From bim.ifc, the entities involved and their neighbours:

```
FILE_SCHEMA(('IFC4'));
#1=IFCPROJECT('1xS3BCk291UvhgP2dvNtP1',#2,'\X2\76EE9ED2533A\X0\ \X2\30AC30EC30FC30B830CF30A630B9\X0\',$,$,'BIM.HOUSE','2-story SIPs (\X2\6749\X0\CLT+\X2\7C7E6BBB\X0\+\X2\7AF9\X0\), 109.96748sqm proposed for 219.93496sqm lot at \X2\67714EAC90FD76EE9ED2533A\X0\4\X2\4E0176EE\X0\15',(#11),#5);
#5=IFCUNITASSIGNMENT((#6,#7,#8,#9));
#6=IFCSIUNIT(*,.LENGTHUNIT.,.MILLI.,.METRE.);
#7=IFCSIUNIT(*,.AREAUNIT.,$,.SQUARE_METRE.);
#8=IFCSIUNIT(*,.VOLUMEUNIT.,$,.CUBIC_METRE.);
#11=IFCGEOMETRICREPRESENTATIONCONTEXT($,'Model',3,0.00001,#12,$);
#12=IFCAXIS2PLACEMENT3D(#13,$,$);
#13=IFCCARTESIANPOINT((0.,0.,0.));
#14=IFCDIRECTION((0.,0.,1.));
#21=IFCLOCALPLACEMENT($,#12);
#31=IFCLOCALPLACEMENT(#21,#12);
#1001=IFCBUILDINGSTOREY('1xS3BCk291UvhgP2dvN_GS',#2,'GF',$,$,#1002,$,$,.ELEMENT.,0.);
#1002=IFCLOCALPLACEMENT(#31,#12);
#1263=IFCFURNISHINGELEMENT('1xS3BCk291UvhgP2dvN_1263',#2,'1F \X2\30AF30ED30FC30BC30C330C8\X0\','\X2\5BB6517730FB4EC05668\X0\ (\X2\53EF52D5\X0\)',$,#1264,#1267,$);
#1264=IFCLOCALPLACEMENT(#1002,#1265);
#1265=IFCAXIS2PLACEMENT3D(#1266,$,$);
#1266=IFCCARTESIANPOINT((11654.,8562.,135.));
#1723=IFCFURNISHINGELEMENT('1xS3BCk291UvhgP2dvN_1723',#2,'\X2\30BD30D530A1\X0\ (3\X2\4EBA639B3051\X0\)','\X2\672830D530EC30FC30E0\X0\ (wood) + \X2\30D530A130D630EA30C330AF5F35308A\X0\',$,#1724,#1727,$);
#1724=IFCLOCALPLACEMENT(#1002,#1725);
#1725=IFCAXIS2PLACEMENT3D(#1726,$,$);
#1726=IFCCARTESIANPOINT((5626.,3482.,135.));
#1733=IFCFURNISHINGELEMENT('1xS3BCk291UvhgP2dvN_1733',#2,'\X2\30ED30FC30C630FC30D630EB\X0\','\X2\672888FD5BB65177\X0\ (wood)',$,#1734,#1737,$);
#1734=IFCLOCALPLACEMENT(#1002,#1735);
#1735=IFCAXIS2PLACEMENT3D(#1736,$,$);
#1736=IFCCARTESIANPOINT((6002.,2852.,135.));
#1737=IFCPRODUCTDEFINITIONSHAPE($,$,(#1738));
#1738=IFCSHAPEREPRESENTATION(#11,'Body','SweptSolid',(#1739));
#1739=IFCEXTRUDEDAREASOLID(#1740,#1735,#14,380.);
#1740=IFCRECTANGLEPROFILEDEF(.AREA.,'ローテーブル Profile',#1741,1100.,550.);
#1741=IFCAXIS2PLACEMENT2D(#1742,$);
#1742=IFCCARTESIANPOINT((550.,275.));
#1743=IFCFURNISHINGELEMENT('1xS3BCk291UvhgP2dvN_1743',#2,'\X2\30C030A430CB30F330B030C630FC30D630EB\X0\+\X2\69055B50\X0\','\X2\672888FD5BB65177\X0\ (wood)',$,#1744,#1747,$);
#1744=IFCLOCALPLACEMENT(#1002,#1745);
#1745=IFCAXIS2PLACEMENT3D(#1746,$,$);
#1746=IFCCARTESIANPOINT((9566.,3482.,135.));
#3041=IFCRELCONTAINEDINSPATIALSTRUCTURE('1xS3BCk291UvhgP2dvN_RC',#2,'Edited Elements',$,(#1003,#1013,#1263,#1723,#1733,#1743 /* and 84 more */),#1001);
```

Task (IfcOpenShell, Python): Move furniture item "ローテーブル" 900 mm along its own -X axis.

```python
import ifcopenshell
import ifcopenshell.api.geometry
import ifcopenshell.util.placement

model = ifcopenshell.open("bim.ifc")

item = model.by_id(1733)
matrix = ifcopenshell.util.placement.get_local_placement(item.ObjectPlacement)
matrix[:3, 3] -= matrix[:3, 0] * 900.0
ifcopenshell.api.geometry.edit_object_placement(model, product=item, matrix=matrix, is_si=False)

print(ifcopenshell.util.placement.get_local_placement(item.ObjectPlacement).round(3) + 0.0)

model.write("bim_rev.ifc")
```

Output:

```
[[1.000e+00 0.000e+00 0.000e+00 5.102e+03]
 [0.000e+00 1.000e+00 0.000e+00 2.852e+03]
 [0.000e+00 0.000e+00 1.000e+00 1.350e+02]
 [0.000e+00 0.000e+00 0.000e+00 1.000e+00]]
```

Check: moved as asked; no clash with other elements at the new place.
